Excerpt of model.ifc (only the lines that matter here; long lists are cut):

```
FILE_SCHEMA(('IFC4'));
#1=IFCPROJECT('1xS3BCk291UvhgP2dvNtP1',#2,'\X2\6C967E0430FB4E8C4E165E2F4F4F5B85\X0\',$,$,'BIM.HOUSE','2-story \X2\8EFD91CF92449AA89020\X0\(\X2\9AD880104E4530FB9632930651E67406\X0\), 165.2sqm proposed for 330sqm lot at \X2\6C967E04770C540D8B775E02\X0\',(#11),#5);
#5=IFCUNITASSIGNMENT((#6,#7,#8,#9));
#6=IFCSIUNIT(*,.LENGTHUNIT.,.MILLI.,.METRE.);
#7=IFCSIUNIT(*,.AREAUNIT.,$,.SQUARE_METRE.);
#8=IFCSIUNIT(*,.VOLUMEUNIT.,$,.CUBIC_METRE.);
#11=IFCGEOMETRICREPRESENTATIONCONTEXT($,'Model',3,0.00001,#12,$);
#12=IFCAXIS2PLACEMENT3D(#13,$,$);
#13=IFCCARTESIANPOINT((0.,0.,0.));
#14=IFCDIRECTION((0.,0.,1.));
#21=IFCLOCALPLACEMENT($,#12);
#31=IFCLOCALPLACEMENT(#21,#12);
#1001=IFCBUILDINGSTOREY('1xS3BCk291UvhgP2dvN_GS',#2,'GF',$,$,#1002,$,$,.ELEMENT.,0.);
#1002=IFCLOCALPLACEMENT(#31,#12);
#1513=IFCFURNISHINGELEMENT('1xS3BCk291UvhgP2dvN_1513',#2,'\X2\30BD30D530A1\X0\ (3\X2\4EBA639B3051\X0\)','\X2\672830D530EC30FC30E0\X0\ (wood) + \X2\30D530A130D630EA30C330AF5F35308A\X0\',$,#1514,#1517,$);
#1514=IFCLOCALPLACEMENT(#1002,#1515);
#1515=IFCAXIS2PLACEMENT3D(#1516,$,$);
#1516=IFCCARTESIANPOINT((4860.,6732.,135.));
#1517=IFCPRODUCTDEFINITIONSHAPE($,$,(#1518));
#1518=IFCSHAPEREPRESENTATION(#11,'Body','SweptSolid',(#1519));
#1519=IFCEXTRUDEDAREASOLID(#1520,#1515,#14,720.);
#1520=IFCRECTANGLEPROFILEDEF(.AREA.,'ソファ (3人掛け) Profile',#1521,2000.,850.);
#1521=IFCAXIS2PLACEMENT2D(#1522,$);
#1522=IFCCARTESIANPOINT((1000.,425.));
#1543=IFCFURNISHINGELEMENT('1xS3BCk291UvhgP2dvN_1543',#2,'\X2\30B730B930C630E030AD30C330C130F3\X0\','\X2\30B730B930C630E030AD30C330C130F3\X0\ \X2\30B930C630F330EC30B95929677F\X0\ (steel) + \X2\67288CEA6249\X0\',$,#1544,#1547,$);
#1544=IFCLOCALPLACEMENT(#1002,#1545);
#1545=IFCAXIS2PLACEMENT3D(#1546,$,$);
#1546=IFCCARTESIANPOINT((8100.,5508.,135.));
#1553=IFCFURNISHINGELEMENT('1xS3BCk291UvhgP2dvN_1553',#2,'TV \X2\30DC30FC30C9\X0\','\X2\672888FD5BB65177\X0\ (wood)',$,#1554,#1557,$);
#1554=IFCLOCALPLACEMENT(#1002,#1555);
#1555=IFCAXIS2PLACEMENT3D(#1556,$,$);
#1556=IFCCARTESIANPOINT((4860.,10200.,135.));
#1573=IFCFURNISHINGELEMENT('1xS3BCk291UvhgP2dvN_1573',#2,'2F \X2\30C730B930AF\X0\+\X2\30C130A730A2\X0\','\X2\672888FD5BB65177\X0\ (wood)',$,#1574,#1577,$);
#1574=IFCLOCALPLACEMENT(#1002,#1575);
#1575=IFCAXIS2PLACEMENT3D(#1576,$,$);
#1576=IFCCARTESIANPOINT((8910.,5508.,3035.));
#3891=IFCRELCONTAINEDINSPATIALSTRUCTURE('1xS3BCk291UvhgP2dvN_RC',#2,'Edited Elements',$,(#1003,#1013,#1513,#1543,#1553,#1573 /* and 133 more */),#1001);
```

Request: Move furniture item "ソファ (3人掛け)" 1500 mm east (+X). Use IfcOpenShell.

```python
import ifcopenshell
import ifcopenshell.api.geometry
import ifcopenshell.util.placement

model = ifcopenshell.open("model.ifc")

item = model.by_guid("1xS3BCk291UvhgP2dvN_1513")
matrix = ifcopenshell.util.placement.get_local_placement(item.ObjectPlacement)
matrix[0, 3] += 1500.0
ifcopenshell.api.geometry.edit_object_placement(model, product=item, matrix=matrix, is_si=False)

print(ifcopenshell.util.placement.get_local_placement(item.ObjectPlacement).round(3) + 0.0)

model.write("model_v2.ifc")
```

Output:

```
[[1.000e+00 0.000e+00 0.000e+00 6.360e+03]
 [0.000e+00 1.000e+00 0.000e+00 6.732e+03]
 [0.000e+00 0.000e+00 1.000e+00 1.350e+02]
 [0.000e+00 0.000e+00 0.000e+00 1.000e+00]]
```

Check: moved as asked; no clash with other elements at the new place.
